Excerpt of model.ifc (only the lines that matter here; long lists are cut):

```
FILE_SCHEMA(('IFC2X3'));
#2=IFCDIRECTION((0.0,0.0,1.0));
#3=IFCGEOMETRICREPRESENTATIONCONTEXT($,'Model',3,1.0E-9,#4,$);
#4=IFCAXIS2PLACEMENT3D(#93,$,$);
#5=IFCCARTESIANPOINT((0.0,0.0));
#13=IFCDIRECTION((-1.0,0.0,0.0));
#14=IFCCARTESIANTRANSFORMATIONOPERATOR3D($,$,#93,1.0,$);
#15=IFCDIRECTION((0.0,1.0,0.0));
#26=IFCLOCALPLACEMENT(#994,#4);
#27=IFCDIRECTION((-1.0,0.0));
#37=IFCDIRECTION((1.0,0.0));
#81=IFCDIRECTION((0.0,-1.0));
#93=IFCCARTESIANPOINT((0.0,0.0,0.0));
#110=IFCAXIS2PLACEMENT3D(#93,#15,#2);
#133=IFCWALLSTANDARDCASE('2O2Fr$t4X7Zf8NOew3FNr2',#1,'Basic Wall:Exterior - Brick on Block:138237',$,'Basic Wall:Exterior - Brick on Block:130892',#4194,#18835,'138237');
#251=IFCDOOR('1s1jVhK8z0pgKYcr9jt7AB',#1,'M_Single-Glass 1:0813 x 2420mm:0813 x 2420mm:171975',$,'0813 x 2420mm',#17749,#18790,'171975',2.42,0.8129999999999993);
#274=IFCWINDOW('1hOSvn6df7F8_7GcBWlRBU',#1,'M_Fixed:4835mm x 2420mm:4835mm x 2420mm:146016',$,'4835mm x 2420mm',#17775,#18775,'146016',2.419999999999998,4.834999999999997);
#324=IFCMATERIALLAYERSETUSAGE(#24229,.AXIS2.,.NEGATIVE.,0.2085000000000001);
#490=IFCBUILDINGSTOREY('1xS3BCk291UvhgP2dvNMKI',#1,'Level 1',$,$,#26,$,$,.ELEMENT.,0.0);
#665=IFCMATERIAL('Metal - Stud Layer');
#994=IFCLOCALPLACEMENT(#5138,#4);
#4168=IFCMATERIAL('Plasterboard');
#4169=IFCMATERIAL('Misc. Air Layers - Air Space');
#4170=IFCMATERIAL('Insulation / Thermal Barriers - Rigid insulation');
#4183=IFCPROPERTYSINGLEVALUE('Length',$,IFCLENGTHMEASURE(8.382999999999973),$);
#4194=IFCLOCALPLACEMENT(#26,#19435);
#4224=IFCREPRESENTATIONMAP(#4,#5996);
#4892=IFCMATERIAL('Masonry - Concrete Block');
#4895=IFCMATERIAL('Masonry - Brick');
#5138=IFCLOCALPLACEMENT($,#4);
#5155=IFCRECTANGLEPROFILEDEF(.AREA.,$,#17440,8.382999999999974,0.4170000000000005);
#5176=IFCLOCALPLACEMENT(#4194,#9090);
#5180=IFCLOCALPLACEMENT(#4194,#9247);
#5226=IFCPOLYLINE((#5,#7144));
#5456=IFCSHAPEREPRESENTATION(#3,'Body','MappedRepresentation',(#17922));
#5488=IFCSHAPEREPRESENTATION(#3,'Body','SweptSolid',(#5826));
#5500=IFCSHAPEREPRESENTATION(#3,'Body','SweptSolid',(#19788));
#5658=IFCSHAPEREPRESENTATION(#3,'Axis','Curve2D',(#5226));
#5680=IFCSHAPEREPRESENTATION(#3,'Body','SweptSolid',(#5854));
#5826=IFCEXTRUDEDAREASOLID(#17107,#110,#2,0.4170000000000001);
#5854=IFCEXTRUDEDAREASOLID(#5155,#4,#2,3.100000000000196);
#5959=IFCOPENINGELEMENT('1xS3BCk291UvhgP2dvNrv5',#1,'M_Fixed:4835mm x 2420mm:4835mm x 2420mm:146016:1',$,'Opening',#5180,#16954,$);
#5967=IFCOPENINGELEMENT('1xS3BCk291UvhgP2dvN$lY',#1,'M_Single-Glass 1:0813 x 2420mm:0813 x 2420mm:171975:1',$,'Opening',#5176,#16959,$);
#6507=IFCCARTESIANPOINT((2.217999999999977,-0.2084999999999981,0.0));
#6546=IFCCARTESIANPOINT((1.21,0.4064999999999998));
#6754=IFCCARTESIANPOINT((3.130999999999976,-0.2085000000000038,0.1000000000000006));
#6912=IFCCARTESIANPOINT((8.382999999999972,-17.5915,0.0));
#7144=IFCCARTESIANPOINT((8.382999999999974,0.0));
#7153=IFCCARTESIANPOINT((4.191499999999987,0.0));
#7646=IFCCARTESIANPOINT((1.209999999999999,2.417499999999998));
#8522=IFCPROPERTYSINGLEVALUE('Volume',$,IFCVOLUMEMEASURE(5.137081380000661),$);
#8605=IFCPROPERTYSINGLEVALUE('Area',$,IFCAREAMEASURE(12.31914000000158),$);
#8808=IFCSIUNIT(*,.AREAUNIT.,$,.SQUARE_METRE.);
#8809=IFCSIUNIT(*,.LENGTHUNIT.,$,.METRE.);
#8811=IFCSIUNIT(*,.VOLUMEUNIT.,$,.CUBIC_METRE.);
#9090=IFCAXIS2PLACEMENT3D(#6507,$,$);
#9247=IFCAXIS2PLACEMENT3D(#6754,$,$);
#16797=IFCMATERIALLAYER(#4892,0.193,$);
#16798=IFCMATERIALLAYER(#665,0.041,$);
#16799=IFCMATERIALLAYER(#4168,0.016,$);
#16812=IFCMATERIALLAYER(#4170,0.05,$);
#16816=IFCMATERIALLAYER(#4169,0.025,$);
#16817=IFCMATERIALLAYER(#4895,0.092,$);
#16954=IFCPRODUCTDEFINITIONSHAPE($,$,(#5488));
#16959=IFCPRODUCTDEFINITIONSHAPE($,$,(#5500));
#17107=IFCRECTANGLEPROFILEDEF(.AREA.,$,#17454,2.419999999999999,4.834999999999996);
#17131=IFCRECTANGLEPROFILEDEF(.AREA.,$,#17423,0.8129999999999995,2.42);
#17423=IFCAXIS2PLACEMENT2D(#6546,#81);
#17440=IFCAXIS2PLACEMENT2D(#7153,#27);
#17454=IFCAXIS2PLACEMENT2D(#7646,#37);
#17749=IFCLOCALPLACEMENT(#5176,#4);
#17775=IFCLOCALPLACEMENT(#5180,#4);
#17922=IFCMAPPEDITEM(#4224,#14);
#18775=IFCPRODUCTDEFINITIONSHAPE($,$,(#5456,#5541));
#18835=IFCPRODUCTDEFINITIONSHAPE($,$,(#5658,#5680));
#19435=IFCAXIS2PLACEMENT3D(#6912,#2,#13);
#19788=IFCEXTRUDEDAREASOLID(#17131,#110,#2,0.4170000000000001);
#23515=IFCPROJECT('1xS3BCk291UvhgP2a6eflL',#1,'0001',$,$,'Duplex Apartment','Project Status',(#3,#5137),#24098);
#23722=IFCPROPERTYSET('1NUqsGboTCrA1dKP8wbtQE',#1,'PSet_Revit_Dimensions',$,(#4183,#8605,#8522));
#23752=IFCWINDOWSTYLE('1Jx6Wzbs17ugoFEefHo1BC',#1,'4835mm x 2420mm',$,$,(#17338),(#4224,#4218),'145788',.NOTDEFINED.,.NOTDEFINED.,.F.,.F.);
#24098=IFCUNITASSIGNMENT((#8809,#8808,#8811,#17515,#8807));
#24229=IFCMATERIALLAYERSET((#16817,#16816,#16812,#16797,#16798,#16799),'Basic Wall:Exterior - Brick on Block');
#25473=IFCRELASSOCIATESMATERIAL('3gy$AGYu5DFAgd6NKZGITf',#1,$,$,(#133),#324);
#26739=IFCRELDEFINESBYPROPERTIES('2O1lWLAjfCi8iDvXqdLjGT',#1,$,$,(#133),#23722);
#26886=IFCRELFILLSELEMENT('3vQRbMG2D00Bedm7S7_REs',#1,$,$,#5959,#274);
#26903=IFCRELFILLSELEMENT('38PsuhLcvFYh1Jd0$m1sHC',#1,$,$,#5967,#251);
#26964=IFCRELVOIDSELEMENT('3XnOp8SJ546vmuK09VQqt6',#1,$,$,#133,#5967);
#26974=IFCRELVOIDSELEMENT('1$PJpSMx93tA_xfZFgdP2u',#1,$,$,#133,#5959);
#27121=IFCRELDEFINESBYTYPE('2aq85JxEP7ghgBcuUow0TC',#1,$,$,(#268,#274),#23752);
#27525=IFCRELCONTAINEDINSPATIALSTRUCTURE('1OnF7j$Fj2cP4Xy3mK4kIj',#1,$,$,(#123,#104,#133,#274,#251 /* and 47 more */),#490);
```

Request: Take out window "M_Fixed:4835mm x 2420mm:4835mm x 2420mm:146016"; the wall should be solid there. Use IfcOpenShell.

```python
import ifcopenshell
import ifcopenshell.api.feature
import ifcopenshell.api.pset
import ifcopenshell.api.root
import ifcopenshell.geom
import ifcopenshell.util.element
import ifcopenshell.util.shape
import ifcopenshell.util.unit

model = ifcopenshell.open("model.ifc")
area_scale = ifcopenshell.util.unit.calculate_unit_scale(model, "AREAUNIT")
volume_scale = ifcopenshell.util.unit.calculate_unit_scale(model, "VOLUMEUNIT")
settings = ifcopenshell.geom.settings()


def volume(element):
    """Net volume in cubic metres, openings subtracted."""
    shape = ifcopenshell.geom.create_shape(settings, element)
    return ifcopenshell.util.shape.get_volume(shape.geometry)


window = model.by_id(274)
opening = window.FillsVoids[0].RelatingOpeningElement
wall = opening.VoidsElements[0].RelatingBuildingElement
before = volume(wall)

ifcopenshell.api.root.remove_product(model, product=window)
ifcopenshell.api.feature.remove_feature(model, feature=opening)

after = volume(wall)
thickness = 0.417  # wall thickness in metres

# Update the wall's stored quantities.
pset = model.by_id(ifcopenshell.util.element.get_pset(wall, "PSet_Revit_Dimensions", should_inherit=False)["id"])
ifcopenshell.api.pset.edit_pset(model, pset=pset, properties={
    "Area": model.create_entity("IfcAreaMeasure", after / thickness / area_scale),
    "Volume": model.create_entity("IfcVolumeMeasure", after / volume_scale),
})

print(f"wall volume {before:.3f} -> {after:.3f} m3")

model.write("model_rev.ifc")
```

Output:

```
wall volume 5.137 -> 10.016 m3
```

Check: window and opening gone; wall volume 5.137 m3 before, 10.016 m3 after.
